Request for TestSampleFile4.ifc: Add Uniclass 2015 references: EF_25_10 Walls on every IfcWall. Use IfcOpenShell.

First a look at what the model holds.

```python
import ifcopenshell

model = ifcopenshell.open("TestSampleFile4.ifc")
print(model.schema)
print("classifications:", [c.Name for c in model.by_type("IfcClassification")])
for ifc_class in ("IfcDoor", "IfcRoof", "IfcStair", "IfcWall", "IfcWindow"):
    print(ifc_class, len(model.by_type(ifc_class)))
```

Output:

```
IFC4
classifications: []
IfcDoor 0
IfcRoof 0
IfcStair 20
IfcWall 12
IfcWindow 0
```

```python
import ifcopenshell
import ifcopenshell.api.classification

model = ifcopenshell.open("TestSampleFile4.ifc")

system = ifcopenshell.api.classification.add_classification(model, classification="Uniclass 2015")

codes = {
    "IfcWall": ("EF_25_10", "Walls"),
}
for ifc_class, (code, name) in codes.items():
    products = model.by_type(ifc_class)
    ifcopenshell.api.classification.add_reference(
        model, products=products, classification=system, identification=code, name=name
    )
    print(code, len(products))

model.write("TestSampleFile4_rev.ifc")
```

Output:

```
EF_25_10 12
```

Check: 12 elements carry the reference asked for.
